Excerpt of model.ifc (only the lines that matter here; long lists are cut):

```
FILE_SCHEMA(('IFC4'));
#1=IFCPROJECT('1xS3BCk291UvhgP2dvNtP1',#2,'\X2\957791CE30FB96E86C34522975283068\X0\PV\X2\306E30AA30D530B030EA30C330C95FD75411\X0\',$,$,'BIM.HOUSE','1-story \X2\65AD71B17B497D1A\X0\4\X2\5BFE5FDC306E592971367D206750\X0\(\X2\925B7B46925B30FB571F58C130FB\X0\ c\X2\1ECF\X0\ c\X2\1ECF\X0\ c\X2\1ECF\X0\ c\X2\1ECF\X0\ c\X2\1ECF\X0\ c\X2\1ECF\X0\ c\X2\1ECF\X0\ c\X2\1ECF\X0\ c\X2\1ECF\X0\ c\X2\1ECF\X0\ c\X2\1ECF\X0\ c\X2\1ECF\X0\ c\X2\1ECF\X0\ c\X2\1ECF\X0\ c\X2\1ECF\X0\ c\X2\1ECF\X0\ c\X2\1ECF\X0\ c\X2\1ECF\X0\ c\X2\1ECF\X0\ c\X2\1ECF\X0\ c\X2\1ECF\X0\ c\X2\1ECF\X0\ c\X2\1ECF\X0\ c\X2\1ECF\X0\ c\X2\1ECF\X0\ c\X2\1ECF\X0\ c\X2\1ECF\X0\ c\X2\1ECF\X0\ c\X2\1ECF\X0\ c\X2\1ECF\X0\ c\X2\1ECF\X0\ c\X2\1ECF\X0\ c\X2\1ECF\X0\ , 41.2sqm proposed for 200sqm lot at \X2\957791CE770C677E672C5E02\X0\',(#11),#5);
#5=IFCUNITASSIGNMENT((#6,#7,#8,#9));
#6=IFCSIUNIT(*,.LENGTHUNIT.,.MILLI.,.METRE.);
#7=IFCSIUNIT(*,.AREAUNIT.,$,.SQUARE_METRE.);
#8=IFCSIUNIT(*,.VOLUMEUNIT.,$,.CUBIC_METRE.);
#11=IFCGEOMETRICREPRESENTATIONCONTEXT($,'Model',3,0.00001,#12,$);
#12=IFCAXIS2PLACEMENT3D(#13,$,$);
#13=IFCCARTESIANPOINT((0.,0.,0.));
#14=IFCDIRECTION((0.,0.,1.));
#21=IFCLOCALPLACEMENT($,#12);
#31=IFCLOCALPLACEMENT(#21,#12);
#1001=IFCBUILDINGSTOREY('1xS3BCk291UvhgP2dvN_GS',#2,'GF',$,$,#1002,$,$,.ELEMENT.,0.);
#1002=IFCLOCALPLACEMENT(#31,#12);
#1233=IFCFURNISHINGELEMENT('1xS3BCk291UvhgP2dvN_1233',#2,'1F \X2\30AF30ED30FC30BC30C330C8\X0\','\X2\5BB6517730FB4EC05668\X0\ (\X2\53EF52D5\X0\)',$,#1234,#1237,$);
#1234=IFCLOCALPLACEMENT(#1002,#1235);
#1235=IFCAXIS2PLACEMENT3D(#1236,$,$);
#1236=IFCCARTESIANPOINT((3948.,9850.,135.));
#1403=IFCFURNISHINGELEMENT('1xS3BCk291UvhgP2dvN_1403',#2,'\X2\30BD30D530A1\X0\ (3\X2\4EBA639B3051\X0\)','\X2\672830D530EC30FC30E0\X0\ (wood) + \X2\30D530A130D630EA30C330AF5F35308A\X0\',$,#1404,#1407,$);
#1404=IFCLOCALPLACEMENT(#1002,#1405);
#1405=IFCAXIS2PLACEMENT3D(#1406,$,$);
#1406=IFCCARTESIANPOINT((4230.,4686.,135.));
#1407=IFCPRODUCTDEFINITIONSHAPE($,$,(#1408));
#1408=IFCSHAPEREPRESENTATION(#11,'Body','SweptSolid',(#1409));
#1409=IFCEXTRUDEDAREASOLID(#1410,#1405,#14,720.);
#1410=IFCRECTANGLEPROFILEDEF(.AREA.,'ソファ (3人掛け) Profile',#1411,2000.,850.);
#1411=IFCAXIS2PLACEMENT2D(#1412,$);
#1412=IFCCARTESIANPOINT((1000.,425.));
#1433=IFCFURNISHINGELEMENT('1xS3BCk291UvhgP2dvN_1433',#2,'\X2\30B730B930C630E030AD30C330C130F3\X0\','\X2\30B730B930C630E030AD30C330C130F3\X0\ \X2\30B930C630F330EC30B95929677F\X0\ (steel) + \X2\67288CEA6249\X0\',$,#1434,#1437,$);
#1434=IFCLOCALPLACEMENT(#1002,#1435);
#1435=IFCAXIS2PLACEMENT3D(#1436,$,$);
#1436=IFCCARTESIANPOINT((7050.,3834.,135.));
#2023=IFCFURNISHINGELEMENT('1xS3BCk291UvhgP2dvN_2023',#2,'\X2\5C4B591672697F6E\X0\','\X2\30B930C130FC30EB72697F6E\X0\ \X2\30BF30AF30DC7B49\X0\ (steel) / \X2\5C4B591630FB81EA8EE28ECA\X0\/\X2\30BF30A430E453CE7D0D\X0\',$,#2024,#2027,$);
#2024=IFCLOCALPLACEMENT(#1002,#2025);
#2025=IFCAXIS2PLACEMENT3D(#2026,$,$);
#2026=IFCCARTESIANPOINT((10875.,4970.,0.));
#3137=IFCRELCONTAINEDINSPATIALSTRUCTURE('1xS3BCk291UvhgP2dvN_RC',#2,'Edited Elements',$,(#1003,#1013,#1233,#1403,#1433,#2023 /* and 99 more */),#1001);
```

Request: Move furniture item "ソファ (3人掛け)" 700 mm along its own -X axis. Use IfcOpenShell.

```python
import ifcopenshell
import ifcopenshell.api.geometry
import ifcopenshell.util.placement
import ifcopenshell.util.unit

model = ifcopenshell.open("model.ifc")
unit_scale = ifcopenshell.util.unit.calculate_unit_scale(model)

item = model.by_guid("1xS3BCk291UvhgP2dvN_1403")
matrix = ifcopenshell.util.placement.get_local_placement(item.ObjectPlacement)
matrix[:3, 3] -= matrix[:3, 0] * 0.7 / unit_scale
ifcopenshell.api.geometry.edit_object_placement(model, product=item, matrix=matrix, is_si=False)

print(ifcopenshell.util.placement.get_local_placement(item.ObjectPlacement).round(3) + 0.0)

model.write("model-out.ifc")
```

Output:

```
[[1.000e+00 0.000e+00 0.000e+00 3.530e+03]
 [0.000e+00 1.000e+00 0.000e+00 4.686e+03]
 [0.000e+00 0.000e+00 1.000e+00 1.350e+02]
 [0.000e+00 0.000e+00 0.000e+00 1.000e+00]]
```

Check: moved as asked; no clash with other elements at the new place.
